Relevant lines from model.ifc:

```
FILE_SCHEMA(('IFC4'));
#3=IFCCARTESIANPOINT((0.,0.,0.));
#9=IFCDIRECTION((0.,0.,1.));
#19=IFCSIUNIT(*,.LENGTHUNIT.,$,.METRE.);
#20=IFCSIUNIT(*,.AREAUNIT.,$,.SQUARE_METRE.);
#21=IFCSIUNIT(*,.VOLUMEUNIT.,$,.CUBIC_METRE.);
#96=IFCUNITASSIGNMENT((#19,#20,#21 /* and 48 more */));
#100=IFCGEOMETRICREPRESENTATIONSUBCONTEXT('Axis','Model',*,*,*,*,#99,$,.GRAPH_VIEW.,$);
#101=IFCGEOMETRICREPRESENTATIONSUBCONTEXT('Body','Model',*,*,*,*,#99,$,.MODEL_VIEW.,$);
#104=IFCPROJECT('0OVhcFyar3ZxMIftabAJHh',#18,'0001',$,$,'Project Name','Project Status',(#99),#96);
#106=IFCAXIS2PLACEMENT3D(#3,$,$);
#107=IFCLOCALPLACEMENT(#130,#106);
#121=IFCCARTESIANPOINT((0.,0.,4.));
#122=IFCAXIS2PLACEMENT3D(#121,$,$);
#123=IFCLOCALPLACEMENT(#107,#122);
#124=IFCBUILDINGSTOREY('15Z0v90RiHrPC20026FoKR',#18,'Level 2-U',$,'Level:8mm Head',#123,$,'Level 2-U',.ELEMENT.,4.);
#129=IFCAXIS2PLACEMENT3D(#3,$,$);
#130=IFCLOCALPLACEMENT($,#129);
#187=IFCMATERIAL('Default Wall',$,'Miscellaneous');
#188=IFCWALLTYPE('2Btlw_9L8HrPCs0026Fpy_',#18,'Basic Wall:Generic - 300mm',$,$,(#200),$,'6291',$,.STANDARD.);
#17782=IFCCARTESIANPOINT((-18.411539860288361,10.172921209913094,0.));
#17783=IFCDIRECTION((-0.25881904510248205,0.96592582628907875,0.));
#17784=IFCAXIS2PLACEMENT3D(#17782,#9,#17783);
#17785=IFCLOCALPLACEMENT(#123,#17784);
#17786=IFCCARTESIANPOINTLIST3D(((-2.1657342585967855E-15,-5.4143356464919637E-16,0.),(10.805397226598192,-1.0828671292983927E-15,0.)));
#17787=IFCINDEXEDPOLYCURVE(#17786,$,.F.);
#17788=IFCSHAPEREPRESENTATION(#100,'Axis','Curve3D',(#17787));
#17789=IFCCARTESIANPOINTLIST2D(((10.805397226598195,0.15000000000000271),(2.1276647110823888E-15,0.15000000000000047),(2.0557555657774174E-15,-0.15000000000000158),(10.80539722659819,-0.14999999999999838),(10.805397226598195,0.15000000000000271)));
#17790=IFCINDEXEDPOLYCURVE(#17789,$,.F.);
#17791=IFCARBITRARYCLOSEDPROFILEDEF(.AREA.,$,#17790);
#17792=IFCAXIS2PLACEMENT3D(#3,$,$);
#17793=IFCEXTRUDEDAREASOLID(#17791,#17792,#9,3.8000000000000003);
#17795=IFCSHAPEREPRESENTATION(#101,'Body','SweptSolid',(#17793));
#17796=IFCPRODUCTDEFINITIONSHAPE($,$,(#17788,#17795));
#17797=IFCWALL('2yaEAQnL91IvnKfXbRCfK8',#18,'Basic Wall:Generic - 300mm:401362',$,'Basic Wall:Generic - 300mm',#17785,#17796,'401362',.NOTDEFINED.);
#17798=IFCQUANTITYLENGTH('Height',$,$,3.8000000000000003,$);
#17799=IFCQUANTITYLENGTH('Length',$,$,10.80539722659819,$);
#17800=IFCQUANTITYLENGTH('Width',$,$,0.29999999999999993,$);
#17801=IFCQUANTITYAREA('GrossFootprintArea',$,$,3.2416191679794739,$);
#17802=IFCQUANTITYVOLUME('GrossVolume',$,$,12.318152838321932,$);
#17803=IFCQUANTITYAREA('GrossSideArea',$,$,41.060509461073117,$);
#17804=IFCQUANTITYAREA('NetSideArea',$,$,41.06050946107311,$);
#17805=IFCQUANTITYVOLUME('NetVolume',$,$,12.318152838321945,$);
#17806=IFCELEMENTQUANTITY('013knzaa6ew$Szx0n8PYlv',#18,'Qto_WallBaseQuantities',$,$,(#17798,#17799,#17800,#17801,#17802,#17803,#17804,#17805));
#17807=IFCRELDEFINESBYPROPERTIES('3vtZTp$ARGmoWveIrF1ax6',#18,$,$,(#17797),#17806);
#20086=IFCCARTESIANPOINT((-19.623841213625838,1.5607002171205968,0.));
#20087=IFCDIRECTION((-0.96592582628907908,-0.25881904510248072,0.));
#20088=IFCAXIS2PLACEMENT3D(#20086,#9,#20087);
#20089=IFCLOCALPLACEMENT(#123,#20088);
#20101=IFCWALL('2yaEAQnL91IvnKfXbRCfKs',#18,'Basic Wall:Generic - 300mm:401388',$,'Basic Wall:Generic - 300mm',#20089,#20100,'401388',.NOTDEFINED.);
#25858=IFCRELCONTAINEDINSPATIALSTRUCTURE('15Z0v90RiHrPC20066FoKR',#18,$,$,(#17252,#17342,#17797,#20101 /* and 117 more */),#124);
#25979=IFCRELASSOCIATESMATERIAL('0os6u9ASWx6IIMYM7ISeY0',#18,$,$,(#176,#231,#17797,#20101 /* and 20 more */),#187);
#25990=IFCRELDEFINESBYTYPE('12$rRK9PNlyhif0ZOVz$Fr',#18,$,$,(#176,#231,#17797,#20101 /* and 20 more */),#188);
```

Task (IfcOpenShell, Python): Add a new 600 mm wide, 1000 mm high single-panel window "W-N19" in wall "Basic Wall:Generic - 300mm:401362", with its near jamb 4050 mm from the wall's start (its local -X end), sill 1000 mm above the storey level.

```python
import numpy as np
import ifcopenshell
import ifcopenshell.api.feature
import ifcopenshell.api.geometry
import ifcopenshell.api.pset
import ifcopenshell.api.root
import ifcopenshell.api.spatial
import ifcopenshell.geom
import ifcopenshell.util.element
import ifcopenshell.util.placement
import ifcopenshell.util.representation
import ifcopenshell.util.shape
import ifcopenshell.util.unit

model = ifcopenshell.open("model.ifc")
unit_scale = ifcopenshell.util.unit.calculate_unit_scale(model)
area_scale = ifcopenshell.util.unit.calculate_unit_scale(model, "AREAUNIT")
volume_scale = ifcopenshell.util.unit.calculate_unit_scale(model, "VOLUMEUNIT")
settings = ifcopenshell.geom.settings()


def volume(element):
    """Net volume in cubic metres, openings subtracted."""
    shape = ifcopenshell.geom.create_shape(settings, element)
    return ifcopenshell.util.shape.get_volume(shape.geometry)


wall = model.by_guid("2yaEAQnL91IvnKfXbRCfK8")
storey = ifcopenshell.util.element.get_container(wall, ifc_class="IfcBuildingStorey")
context = ifcopenshell.util.representation.get_context(model, "Model", "Body", "MODEL_VIEW")
before = volume(wall)

width, height, from_end, sill = 0.6, 1, 4.05, 1  # metres

# The wall runs along its own X axis, and the end named is its -X end.
wall_shape = ifcopenshell.geom.create_shape(settings, wall)
x, y, z = ifcopenshell.util.shape.get_vertices(wall_shape.geometry).T
start = x.min() + from_end
face, thickness = float(y.min()), float(y.max() - y.min())
wall_matrix = ifcopenshell.util.placement.get_local_placement(wall.ObjectPlacement)
level = ifcopenshell.util.placement.get_local_placement(storey.ObjectPlacement)[2, 3]


def in_wall(x, y):
    """Placement at x, y metres in the wall's axes, at sill height."""
    matrix = wall_matrix.copy()
    matrix[:, 3] = wall_matrix @ np.array([x / unit_scale, y / unit_scale, 0.0, 1.0])
    matrix[2, 3] = level + sill / unit_scale
    return matrix


# Opening: a box that overshoots both wall faces by 50 mm.
opening = ifcopenshell.api.root.create_entity(model, ifc_class="IfcOpeningElement", predefined_type="OPENING")
box = ifcopenshell.api.geometry.add_wall_representation(
    model, context=context, length=width, height=height, thickness=thickness + 0.1
)
ifcopenshell.api.geometry.assign_representation(model, product=opening, representation=box)
ifcopenshell.api.geometry.edit_object_placement(model, product=opening, matrix=in_wall(start, face - 0.05), is_si=False)
ifcopenshell.api.feature.add_feature(model, feature=opening, element=wall)

window = ifcopenshell.api.root.create_entity(model, ifc_class="IfcWindow", name="W-N19", predefined_type="WINDOW")
window.OverallWidth, window.OverallHeight = width / unit_scale, height / unit_scale
window.PartitioningType = "SINGLE_PANEL"
body = ifcopenshell.api.geometry.add_window_representation(
    model,
    context=context,
    overall_width=window.OverallWidth,
    overall_height=window.OverallHeight,
    partition_type="SINGLE_PANEL",
)
ifcopenshell.api.geometry.assign_representation(model, product=window, representation=body)
ifcopenshell.api.spatial.assign_container(model, products=[window], relating_structure=storey)
ifcopenshell.api.feature.add_filling(model, opening=opening, element=window)

# Centre the window in the wall's thickness.
ifcopenshell.api.geometry.edit_object_placement(model, product=window, matrix=in_wall(start, face), is_si=False)
window_shape = ifcopenshell.geom.create_shape(settings, window)
depth = ifcopenshell.util.shape.get_vertices(window_shape.geometry)[:, 1]
offset = face + thickness / 2 - (depth.min() + depth.max()) / 2
ifcopenshell.api.geometry.edit_object_placement(model, product=window, matrix=in_wall(start, offset), is_si=False)

after = volume(wall)

# Update the wall's stored quantities.
qto = model.by_id(ifcopenshell.util.element.get_pset(wall, "Qto_WallBaseQuantities", should_inherit=False)["id"])
ifcopenshell.api.pset.edit_qto(model, qto=qto, properties={
    "NetSideArea": after / thickness / area_scale,
    "NetVolume": after / volume_scale,
})

print(f"wall volume {before:.3f} -> {after:.3f} m3")

model.write("model_updated.ifc")
```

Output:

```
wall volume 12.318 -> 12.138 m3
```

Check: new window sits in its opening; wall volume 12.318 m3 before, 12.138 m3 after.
